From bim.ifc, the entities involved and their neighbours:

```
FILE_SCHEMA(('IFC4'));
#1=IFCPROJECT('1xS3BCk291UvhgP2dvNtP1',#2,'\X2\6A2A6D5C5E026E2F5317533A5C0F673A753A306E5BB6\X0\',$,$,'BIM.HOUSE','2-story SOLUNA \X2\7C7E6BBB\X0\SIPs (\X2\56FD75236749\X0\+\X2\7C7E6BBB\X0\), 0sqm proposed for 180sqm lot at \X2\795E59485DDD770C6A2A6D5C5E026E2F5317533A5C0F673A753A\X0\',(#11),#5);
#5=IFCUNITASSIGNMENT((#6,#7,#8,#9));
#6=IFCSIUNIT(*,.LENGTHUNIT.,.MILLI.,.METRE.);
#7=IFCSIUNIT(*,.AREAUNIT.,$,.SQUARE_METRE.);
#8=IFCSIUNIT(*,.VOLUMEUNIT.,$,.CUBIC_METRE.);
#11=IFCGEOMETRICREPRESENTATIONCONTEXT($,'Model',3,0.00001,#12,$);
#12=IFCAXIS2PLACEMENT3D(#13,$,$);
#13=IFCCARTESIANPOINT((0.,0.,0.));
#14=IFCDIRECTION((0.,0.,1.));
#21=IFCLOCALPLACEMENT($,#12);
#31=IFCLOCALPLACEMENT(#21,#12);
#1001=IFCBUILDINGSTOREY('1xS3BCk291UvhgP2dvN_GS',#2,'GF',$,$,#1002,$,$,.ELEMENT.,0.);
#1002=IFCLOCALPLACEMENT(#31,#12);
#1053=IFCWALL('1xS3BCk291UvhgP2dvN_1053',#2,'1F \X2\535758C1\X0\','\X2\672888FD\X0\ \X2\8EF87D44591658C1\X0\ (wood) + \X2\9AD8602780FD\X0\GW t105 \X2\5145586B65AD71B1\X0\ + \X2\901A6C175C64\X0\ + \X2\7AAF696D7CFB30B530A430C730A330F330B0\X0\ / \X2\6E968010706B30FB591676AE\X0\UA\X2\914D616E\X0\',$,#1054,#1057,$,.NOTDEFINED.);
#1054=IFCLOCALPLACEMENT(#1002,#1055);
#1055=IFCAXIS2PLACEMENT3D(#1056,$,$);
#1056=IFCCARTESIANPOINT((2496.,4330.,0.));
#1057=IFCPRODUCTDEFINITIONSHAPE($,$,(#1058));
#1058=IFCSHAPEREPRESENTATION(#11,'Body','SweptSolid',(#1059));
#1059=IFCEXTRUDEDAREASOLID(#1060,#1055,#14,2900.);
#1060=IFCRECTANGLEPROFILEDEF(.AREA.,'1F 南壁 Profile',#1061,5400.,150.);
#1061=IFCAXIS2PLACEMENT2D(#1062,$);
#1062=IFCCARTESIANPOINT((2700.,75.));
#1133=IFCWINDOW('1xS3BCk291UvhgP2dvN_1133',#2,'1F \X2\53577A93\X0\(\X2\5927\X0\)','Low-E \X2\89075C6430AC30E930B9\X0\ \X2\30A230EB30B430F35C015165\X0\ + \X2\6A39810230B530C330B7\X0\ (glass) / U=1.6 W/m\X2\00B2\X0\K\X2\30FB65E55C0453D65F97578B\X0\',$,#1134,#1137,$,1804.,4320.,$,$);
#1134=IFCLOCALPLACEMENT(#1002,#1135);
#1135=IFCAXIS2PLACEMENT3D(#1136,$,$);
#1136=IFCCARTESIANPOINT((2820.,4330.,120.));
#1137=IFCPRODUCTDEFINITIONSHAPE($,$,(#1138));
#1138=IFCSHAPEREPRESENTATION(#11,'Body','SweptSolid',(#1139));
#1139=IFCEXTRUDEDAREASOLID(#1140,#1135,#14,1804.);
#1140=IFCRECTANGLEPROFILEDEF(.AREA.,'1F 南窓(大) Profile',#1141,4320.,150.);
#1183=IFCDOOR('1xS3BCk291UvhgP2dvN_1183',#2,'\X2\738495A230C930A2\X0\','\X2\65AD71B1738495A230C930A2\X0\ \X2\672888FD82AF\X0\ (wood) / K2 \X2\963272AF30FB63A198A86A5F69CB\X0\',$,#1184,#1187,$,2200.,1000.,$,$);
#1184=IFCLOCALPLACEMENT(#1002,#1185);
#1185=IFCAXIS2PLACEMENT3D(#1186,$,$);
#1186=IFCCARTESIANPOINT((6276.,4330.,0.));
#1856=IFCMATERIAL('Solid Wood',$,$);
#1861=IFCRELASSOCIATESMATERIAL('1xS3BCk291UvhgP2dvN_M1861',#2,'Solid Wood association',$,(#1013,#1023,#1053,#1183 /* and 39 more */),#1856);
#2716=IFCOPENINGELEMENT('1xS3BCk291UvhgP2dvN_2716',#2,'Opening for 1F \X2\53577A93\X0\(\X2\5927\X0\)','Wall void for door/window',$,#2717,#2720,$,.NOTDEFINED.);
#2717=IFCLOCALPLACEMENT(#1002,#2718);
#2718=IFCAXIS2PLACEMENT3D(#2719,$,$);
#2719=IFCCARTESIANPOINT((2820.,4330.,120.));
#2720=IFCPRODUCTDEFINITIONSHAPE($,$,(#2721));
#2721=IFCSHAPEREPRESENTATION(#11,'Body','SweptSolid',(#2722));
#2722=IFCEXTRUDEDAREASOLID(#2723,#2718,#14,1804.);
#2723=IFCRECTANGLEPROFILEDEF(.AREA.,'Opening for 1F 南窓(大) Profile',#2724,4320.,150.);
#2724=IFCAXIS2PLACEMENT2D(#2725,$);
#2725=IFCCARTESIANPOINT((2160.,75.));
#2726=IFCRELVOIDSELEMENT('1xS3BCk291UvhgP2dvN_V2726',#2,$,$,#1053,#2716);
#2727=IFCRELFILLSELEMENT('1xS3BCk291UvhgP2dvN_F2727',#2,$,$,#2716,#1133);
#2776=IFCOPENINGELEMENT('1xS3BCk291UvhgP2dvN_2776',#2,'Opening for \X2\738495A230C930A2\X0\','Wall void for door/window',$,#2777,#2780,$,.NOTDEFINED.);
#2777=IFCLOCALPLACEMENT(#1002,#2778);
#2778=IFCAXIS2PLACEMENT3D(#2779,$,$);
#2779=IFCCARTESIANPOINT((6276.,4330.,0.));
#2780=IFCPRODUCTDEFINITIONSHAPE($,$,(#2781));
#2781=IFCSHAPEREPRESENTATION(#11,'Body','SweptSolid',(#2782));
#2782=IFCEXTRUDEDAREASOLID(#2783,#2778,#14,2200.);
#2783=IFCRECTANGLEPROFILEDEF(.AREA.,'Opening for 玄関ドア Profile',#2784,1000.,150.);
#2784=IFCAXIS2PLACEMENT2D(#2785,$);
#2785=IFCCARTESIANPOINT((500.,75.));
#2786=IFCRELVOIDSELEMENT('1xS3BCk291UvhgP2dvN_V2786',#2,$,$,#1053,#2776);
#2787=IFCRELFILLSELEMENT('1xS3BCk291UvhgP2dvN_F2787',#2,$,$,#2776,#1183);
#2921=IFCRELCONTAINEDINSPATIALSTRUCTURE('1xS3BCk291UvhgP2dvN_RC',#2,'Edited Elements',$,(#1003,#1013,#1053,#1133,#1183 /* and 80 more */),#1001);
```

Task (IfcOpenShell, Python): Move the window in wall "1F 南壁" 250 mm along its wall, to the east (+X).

```python
import ifcopenshell
import ifcopenshell.api.geometry
import ifcopenshell.util.placement
import ifcopenshell.util.unit

model = ifcopenshell.open("bim.ifc")
unit_scale = ifcopenshell.util.unit.calculate_unit_scale(model)

window = model.by_guid("1xS3BCk291UvhgP2dvN_1133")
opening = window.FillsVoids[0].RelatingOpeningElement
wall = opening.VoidsElements[0].RelatingBuildingElement

wall_matrix = ifcopenshell.util.placement.get_local_placement(wall.ObjectPlacement)
shift = wall_matrix[:3, 0] * 0.25 / unit_scale
before = ifcopenshell.util.placement.get_local_placement(window.ObjectPlacement)[:3, 3].copy()

# The window is not placed relative to its opening, so move both.
for product in (opening, window):
    matrix = ifcopenshell.util.placement.get_local_placement(product.ObjectPlacement)
    matrix[:3, 3] += shift
    ifcopenshell.api.geometry.edit_object_placement(model, product=product, matrix=matrix, is_si=False)

after = ifcopenshell.util.placement.get_local_placement(window.ObjectPlacement)[:3, 3]
print("window moved by", (after - before).round(3) + 0.0)

model.write("bim-out.ifc")
```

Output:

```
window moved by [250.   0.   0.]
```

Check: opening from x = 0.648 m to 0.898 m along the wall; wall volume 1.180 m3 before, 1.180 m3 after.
